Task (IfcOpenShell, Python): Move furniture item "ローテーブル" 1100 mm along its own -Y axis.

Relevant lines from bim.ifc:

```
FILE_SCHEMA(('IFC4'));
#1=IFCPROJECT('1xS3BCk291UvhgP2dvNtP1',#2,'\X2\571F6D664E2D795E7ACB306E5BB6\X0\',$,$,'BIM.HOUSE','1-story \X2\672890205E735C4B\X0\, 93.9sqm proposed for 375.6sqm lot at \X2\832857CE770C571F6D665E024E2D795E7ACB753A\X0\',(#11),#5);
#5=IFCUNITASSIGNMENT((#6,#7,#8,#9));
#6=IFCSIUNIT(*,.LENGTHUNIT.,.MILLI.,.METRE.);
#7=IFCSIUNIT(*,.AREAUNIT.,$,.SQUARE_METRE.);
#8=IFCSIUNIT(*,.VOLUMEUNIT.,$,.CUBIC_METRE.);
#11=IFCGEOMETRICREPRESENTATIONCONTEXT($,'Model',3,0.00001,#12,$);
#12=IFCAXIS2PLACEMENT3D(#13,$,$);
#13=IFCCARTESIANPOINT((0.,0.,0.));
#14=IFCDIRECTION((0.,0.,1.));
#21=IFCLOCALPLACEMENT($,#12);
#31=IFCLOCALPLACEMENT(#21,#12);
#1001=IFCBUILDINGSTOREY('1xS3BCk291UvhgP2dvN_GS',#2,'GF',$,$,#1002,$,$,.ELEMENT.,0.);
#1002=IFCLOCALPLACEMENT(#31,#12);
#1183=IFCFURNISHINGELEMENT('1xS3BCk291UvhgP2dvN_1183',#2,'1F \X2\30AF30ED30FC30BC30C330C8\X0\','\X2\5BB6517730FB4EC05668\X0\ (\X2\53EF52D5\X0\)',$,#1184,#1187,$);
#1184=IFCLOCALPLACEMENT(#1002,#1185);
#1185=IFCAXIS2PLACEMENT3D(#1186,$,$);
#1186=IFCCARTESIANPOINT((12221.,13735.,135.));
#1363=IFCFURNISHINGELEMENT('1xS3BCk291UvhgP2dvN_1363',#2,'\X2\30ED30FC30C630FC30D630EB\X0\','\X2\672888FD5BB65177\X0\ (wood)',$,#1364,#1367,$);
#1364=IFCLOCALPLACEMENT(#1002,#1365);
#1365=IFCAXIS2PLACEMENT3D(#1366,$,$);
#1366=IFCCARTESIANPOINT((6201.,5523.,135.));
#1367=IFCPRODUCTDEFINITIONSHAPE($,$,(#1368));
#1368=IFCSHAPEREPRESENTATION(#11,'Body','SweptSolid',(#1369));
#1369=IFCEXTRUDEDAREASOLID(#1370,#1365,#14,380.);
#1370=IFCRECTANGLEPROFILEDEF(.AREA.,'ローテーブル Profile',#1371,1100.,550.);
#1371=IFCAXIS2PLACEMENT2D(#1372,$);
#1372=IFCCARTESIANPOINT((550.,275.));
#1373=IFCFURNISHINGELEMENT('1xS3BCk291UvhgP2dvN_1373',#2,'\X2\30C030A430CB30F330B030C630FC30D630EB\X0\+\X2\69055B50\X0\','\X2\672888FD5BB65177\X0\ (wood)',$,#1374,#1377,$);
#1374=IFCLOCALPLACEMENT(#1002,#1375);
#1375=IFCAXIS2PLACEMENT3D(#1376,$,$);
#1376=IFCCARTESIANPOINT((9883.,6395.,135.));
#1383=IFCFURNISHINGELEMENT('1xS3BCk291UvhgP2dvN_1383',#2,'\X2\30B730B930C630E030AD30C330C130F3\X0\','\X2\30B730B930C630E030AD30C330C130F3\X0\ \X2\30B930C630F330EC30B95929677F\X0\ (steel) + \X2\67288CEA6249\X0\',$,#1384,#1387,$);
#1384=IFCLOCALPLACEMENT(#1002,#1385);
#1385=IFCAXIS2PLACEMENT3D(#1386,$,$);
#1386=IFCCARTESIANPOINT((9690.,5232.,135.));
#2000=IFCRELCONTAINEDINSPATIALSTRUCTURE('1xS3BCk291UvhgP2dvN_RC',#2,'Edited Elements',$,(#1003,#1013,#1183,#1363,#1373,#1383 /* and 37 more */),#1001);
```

```python
import ifcopenshell
import ifcopenshell.api.geometry
import ifcopenshell.util.placement
import ifcopenshell.util.unit

model = ifcopenshell.open("bim.ifc")
unit_scale = ifcopenshell.util.unit.calculate_unit_scale(model)

item = model.by_id(1363)
matrix = ifcopenshell.util.placement.get_local_placement(item.ObjectPlacement)
matrix[:3, 3] -= matrix[:3, 1] * 1.1 / unit_scale
ifcopenshell.api.geometry.edit_object_placement(model, product=item, matrix=matrix, is_si=False)

print(ifcopenshell.util.placement.get_local_placement(item.ObjectPlacement).round(3) + 0.0)

model.write("bim_edited.ifc")
```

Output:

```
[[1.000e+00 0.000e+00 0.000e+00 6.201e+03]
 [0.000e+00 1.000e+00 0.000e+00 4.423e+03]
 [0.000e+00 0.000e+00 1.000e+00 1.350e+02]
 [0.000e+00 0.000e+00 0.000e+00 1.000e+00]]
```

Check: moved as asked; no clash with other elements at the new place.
